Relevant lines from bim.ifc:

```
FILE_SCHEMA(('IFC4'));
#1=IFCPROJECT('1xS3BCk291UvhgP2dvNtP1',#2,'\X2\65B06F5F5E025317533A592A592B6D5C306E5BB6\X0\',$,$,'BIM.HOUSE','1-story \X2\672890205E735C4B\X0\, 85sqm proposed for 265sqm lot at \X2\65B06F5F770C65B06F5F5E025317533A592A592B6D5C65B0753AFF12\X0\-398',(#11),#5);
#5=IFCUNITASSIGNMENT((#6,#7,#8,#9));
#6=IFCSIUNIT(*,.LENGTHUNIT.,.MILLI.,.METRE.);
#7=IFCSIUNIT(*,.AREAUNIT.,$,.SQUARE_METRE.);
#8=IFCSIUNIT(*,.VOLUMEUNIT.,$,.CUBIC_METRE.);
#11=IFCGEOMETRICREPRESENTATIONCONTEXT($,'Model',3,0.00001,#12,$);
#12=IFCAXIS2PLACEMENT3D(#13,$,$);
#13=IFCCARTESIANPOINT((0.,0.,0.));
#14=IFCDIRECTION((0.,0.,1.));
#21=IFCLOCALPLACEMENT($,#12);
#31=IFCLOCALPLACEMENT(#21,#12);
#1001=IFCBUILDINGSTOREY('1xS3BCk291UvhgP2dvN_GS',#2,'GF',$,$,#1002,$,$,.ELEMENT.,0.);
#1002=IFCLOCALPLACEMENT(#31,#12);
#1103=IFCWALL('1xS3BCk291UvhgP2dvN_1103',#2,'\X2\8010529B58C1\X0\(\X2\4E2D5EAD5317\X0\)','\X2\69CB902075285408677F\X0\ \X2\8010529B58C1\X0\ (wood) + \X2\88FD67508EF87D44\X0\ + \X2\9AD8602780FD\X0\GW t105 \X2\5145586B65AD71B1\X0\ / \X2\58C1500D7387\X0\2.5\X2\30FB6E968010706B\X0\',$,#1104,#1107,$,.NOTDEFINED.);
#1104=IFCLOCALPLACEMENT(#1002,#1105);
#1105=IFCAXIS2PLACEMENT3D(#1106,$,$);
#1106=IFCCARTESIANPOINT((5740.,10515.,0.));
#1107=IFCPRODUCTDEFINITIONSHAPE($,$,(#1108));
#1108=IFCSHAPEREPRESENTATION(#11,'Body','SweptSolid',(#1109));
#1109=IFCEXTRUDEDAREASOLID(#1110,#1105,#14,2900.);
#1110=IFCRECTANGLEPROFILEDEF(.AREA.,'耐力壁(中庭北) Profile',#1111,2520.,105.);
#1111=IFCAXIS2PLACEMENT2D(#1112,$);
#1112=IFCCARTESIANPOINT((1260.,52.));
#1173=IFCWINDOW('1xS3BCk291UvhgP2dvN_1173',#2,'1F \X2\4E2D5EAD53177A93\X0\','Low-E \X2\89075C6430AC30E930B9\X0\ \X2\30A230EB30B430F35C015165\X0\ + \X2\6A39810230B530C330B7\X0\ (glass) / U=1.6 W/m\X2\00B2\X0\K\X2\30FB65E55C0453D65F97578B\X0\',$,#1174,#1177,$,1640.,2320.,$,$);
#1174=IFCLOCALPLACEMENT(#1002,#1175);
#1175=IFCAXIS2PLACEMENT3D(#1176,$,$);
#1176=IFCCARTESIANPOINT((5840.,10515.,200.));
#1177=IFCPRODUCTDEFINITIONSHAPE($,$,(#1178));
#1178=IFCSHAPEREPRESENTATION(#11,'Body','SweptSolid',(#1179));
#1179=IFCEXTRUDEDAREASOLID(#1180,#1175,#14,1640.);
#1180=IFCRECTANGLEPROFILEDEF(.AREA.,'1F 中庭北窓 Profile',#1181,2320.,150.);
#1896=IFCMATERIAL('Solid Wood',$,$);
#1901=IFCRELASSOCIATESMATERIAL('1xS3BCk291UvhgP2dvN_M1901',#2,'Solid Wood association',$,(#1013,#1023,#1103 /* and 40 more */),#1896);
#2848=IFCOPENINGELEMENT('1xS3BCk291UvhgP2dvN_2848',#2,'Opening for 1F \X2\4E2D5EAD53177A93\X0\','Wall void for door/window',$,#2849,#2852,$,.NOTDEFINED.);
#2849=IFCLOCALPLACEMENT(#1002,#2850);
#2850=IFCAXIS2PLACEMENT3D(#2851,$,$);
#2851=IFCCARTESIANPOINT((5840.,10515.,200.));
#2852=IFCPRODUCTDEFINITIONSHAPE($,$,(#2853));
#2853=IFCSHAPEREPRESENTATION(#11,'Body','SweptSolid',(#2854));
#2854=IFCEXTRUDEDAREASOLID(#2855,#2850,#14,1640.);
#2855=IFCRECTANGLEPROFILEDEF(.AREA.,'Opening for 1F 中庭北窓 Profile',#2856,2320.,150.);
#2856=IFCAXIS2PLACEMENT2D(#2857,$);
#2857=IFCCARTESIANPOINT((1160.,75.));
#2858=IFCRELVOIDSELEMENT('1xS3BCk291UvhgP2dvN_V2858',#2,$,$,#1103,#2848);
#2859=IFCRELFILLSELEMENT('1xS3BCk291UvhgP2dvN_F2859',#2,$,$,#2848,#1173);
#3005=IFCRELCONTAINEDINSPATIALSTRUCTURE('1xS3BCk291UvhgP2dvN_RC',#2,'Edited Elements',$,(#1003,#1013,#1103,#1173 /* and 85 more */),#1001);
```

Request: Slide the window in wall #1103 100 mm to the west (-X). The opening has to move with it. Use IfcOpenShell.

```python
import ifcopenshell
import ifcopenshell.api.geometry
import ifcopenshell.util.placement

model = ifcopenshell.open("bim.ifc")

window = model.by_id(1173)
opening = window.FillsVoids[0].RelatingOpeningElement
wall = opening.VoidsElements[0].RelatingBuildingElement

wall_matrix = ifcopenshell.util.placement.get_local_placement(wall.ObjectPlacement)
shift = wall_matrix[:3, 0] * -100.0
before = ifcopenshell.util.placement.get_local_placement(window.ObjectPlacement)[:3, 3].copy()

# The window is not placed relative to its opening, so move both.
for product in (opening, window):
    matrix = ifcopenshell.util.placement.get_local_placement(product.ObjectPlacement)
    matrix[:3, 3] += shift
    ifcopenshell.api.geometry.edit_object_placement(model, product=product, matrix=matrix, is_si=False)

after = ifcopenshell.util.placement.get_local_placement(window.ObjectPlacement)[:3, 3]
print("window moved by", (after - before).round(3) + 0.0)

model.write("bim_v2.ifc")
```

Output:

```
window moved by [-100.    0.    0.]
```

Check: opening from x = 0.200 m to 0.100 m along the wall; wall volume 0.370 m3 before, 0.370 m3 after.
